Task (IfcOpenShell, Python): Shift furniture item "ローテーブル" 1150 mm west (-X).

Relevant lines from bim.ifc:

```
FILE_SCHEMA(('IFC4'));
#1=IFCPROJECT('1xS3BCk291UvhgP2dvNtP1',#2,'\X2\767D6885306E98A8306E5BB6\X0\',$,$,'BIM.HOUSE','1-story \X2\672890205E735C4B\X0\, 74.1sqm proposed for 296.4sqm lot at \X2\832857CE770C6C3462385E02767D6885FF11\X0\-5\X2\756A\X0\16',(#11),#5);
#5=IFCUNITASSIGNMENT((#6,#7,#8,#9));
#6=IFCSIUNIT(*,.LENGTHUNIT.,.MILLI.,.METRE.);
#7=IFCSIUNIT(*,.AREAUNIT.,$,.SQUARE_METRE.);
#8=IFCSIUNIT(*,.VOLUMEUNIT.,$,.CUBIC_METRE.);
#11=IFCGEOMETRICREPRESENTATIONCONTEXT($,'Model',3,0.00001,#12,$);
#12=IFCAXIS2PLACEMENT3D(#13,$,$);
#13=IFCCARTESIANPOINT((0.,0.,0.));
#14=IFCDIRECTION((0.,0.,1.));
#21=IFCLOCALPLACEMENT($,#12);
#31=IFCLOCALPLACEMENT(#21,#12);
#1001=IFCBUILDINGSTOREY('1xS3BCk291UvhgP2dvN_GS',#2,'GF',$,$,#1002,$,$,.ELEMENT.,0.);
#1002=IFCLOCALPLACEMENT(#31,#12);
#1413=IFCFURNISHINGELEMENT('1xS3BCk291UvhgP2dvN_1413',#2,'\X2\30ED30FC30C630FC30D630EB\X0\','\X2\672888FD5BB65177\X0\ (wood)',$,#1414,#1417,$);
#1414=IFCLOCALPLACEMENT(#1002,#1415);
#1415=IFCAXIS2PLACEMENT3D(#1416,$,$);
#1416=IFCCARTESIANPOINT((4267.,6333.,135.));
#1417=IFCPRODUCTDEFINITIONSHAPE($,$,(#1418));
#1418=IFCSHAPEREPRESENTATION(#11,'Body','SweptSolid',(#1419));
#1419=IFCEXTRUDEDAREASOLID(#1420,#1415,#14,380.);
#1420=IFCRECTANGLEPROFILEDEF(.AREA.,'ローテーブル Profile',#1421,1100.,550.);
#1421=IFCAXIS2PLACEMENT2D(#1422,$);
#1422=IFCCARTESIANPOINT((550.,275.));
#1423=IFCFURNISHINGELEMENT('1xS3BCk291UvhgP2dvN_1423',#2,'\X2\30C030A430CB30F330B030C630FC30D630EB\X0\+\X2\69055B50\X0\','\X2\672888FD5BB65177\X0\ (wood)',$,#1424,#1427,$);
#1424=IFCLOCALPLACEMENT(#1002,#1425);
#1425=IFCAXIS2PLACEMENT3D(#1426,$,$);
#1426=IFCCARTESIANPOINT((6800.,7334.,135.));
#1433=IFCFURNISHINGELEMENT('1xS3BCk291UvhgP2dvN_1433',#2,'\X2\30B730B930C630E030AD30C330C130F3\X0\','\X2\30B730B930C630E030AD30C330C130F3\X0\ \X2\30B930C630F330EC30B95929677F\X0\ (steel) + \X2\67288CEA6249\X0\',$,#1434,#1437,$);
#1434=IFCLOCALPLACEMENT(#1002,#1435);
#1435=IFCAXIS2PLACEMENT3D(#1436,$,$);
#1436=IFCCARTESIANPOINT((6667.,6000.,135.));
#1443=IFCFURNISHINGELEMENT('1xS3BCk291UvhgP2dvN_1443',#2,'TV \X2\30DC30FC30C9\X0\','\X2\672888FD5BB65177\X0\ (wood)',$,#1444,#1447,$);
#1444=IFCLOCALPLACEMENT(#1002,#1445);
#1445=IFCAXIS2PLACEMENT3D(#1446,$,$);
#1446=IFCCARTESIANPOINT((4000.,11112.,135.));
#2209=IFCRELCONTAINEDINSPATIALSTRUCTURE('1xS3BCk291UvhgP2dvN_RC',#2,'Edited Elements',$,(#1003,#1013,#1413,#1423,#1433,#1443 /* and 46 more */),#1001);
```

```python
import ifcopenshell
import ifcopenshell.api.geometry
import ifcopenshell.util.placement

model = ifcopenshell.open("bim.ifc")

item = model.by_guid("1xS3BCk291UvhgP2dvN_1413")
matrix = ifcopenshell.util.placement.get_local_placement(item.ObjectPlacement)
matrix[0, 3] -= 1150.0
ifcopenshell.api.geometry.edit_object_placement(model, product=item, matrix=matrix, is_si=False)

print(ifcopenshell.util.placement.get_local_placement(item.ObjectPlacement).round(3) + 0.0)

model.write("bim_edited.ifc")
```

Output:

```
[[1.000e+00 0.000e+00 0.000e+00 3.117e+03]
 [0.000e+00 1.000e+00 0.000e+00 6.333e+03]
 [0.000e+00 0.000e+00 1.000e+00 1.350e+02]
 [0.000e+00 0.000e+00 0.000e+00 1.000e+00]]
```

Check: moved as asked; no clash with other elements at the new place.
